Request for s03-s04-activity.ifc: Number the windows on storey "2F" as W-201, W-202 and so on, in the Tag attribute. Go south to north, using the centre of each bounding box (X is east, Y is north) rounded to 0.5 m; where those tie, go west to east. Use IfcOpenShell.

First a look at what the model holds.

```python
import ifcopenshell
import ifcopenshell.util.element
import ifcopenshell.util.placement

model = ifcopenshell.open("s03-s04-activity.ifc")
print(model.schema)
storey = next(s for s in model.by_type("IfcBuildingStorey") if s.Name == "2F")
windows = [e for e in ifcopenshell.util.element.get_decomposition(storey) if e.is_a("IfcWindow")]
for e in sorted(windows, key=lambda e: e.id()):
    origin = ifcopenshell.util.placement.get_local_placement(e.ObjectPlacement)[:3, 3]
    print(e.id(), e.Tag, e.Name, origin.round(2) + 0.0, sep=" | ")
```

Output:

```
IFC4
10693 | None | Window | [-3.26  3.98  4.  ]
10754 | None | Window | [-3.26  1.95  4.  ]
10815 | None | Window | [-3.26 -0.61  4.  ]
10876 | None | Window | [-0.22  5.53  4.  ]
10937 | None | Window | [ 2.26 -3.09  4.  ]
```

```python
import ifcopenshell
import ifcopenshell.geom
import ifcopenshell.util.element
import ifcopenshell.util.shape

model = ifcopenshell.open("s03-s04-activity.ifc")
settings = ifcopenshell.geom.settings()
settings.set("use-world-coords", True)


def centre(element):
    shape = ifcopenshell.geom.create_shape(settings, element)
    return ifcopenshell.util.shape.get_bbox_centroid(shape.geometry)


storey = next(s for s in model.by_type("IfcBuildingStorey") if s.Name == "2F")
windows = [e for e in ifcopenshell.util.element.get_decomposition(storey) if e.is_a("IfcWindow")]

# Insertion points can sit at a corner or the storey origin, so sort by the geometry (in metres).
centres = {e: centre(e) for e in windows}
windows.sort(key=lambda e: (round(centres[e][1] / 0.5), centres[e][0]))

for i, e in enumerate(windows, start=1):
    number = f"W-2{i:02d}"
    e.Tag = number
    print(e.id(), number)

model.write("s03-s04-activity_rev.ifc")
```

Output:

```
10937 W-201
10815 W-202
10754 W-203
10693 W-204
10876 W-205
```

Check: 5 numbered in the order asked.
